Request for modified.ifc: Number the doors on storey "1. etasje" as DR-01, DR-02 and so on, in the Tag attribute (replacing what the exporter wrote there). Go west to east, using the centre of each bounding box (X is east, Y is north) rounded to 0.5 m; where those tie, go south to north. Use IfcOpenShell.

First a look at what the model holds.

```python
import ifcopenshell
import ifcopenshell.util.element
import ifcopenshell.util.placement

model = ifcopenshell.open("modified.ifc")
print(model.schema)
storey = next(s for s in model.by_type("IfcBuildingStorey") if s.Name == "1. etasje")
doors = [e for e in ifcopenshell.util.element.get_decomposition(storey) if e.is_a("IfcDoor")]
for e in sorted(doors, key=lambda e: e.id()):
    origin = ifcopenshell.util.placement.get_local_placement(e.ObjectPlacement)[:3, 3]
    print(e.id(), e.Tag, e.Name, origin.round(2) + 0.0, sep=" | ")
```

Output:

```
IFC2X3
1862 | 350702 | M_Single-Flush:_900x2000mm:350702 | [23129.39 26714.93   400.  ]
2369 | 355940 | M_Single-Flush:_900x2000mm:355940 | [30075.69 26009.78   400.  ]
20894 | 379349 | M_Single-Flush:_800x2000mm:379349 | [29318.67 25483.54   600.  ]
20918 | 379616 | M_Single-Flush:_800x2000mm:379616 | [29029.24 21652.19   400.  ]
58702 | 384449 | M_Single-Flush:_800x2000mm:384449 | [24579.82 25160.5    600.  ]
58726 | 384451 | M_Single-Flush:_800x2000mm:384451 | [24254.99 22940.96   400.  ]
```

```python
import ifcopenshell
import ifcopenshell.geom
import ifcopenshell.util.element
import ifcopenshell.util.shape

model = ifcopenshell.open("modified.ifc")
settings = ifcopenshell.geom.settings()
settings.set("use-world-coords", True)


def centre(element):
    shape = ifcopenshell.geom.create_shape(settings, element)
    return ifcopenshell.util.shape.get_bbox_centroid(shape.geometry)


storey = next(s for s in model.by_type("IfcBuildingStorey") if s.Name == "1. etasje")
doors = [e for e in ifcopenshell.util.element.get_decomposition(storey) if e.is_a("IfcDoor")]

# Insertion points can sit at a corner or the storey origin, so sort by the geometry (in metres).
centres = {e: centre(e) for e in doors}
doors.sort(key=lambda e: (round(centres[e][0] / 0.5), centres[e][1]))

for i, e in enumerate(doors, start=1):
    number = f"DR-{i:02d}"
    e.Tag = number
    print(e.id(), number)

model.write("modified_edited.ifc")
```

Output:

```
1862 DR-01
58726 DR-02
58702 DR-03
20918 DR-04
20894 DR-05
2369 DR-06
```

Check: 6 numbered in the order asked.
